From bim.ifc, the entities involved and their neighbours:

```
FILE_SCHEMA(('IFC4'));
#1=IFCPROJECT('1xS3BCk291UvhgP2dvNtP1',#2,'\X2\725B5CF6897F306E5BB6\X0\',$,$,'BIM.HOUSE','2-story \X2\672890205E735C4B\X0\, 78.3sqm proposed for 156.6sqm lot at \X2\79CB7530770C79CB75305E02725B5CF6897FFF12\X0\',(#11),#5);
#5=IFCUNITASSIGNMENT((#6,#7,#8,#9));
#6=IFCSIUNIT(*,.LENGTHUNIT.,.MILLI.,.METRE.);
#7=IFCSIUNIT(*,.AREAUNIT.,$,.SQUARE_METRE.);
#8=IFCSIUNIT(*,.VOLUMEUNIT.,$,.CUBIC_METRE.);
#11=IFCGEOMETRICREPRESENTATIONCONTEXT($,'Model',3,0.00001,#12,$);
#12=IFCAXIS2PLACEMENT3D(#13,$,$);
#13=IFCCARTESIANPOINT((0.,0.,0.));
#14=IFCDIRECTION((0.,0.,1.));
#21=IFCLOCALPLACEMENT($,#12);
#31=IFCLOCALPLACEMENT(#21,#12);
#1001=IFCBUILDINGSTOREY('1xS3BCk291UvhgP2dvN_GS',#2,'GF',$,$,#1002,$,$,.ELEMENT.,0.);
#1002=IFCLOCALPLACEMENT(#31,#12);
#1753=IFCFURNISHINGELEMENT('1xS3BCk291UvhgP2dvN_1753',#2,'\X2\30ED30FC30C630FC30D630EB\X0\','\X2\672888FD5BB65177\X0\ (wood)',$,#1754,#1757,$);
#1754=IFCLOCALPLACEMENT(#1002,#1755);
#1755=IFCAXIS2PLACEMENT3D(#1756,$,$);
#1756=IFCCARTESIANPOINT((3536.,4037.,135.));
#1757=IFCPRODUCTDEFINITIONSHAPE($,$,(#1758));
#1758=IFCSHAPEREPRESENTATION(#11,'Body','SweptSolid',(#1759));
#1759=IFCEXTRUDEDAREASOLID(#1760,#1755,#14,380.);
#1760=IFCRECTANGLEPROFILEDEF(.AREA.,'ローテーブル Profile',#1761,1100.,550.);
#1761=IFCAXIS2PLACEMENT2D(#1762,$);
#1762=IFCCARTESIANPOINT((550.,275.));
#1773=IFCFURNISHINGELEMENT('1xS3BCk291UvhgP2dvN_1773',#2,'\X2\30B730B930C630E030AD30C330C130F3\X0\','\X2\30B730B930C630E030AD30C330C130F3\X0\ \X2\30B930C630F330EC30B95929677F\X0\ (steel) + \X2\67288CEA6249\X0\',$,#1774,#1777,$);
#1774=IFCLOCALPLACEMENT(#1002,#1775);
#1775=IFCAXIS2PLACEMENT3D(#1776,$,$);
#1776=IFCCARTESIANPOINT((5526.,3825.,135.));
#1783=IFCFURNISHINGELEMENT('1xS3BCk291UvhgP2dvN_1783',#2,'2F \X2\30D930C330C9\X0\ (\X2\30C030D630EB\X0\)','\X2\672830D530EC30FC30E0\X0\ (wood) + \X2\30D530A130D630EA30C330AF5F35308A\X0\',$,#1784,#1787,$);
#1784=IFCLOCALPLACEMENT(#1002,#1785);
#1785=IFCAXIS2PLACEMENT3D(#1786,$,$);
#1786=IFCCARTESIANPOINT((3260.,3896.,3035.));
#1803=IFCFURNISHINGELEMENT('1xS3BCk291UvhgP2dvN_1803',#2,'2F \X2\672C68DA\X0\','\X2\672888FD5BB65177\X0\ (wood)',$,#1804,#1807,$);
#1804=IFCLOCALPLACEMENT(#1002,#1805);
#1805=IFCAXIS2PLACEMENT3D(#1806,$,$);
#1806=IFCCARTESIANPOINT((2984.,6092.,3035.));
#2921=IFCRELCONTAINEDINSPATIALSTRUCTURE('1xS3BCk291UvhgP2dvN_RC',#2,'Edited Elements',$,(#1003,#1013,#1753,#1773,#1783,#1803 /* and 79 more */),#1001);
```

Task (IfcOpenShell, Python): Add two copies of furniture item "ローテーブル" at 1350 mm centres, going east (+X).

```python
import numpy as np
import ifcopenshell
import ifcopenshell.api.geometry
import ifcopenshell.api.root
import ifcopenshell.util.element
import ifcopenshell.util.placement

model = ifcopenshell.open("bim.ifc")


def reuse_history(source, copy):
    """copy_class also copies each property set's owner history, people and application; keep the originals."""
    for rel in copy.IsDefinedBy:
        if rel.is_a("IfcRelDefinesByProperties") and (history := rel.RelatingPropertyDefinition.OwnerHistory):
            rel.RelatingPropertyDefinition.OwnerHistory = source.OwnerHistory
            ifcopenshell.util.element.remove_deep2(model, history)


source = model.by_guid("1xS3BCk291UvhgP2dvN_1753")
base = ifcopenshell.util.placement.get_local_placement(source.ObjectPlacement)
step = np.array([1.0, 0.0, 0.0]) * 1350.0

for i in range(1, 3):
    copy = ifcopenshell.api.root.copy_class(model, product=source)
    copy.Representation = ifcopenshell.util.element.copy_deep(
        model, source.Representation, exclude=["IfcGeometricRepresentationContext", "IfcRepresentationMap"]
    )
    reuse_history(source, copy)
    matrix = base.copy()
    matrix[:3, 3] += i * step
    print("added at", matrix[:3, 3].round(3) + 0.0)
    ifcopenshell.api.geometry.edit_object_placement(model, product=copy, matrix=matrix, is_si=False)

model.write("bim_edited.ifc")
```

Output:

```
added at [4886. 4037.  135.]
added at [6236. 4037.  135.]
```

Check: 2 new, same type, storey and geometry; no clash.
